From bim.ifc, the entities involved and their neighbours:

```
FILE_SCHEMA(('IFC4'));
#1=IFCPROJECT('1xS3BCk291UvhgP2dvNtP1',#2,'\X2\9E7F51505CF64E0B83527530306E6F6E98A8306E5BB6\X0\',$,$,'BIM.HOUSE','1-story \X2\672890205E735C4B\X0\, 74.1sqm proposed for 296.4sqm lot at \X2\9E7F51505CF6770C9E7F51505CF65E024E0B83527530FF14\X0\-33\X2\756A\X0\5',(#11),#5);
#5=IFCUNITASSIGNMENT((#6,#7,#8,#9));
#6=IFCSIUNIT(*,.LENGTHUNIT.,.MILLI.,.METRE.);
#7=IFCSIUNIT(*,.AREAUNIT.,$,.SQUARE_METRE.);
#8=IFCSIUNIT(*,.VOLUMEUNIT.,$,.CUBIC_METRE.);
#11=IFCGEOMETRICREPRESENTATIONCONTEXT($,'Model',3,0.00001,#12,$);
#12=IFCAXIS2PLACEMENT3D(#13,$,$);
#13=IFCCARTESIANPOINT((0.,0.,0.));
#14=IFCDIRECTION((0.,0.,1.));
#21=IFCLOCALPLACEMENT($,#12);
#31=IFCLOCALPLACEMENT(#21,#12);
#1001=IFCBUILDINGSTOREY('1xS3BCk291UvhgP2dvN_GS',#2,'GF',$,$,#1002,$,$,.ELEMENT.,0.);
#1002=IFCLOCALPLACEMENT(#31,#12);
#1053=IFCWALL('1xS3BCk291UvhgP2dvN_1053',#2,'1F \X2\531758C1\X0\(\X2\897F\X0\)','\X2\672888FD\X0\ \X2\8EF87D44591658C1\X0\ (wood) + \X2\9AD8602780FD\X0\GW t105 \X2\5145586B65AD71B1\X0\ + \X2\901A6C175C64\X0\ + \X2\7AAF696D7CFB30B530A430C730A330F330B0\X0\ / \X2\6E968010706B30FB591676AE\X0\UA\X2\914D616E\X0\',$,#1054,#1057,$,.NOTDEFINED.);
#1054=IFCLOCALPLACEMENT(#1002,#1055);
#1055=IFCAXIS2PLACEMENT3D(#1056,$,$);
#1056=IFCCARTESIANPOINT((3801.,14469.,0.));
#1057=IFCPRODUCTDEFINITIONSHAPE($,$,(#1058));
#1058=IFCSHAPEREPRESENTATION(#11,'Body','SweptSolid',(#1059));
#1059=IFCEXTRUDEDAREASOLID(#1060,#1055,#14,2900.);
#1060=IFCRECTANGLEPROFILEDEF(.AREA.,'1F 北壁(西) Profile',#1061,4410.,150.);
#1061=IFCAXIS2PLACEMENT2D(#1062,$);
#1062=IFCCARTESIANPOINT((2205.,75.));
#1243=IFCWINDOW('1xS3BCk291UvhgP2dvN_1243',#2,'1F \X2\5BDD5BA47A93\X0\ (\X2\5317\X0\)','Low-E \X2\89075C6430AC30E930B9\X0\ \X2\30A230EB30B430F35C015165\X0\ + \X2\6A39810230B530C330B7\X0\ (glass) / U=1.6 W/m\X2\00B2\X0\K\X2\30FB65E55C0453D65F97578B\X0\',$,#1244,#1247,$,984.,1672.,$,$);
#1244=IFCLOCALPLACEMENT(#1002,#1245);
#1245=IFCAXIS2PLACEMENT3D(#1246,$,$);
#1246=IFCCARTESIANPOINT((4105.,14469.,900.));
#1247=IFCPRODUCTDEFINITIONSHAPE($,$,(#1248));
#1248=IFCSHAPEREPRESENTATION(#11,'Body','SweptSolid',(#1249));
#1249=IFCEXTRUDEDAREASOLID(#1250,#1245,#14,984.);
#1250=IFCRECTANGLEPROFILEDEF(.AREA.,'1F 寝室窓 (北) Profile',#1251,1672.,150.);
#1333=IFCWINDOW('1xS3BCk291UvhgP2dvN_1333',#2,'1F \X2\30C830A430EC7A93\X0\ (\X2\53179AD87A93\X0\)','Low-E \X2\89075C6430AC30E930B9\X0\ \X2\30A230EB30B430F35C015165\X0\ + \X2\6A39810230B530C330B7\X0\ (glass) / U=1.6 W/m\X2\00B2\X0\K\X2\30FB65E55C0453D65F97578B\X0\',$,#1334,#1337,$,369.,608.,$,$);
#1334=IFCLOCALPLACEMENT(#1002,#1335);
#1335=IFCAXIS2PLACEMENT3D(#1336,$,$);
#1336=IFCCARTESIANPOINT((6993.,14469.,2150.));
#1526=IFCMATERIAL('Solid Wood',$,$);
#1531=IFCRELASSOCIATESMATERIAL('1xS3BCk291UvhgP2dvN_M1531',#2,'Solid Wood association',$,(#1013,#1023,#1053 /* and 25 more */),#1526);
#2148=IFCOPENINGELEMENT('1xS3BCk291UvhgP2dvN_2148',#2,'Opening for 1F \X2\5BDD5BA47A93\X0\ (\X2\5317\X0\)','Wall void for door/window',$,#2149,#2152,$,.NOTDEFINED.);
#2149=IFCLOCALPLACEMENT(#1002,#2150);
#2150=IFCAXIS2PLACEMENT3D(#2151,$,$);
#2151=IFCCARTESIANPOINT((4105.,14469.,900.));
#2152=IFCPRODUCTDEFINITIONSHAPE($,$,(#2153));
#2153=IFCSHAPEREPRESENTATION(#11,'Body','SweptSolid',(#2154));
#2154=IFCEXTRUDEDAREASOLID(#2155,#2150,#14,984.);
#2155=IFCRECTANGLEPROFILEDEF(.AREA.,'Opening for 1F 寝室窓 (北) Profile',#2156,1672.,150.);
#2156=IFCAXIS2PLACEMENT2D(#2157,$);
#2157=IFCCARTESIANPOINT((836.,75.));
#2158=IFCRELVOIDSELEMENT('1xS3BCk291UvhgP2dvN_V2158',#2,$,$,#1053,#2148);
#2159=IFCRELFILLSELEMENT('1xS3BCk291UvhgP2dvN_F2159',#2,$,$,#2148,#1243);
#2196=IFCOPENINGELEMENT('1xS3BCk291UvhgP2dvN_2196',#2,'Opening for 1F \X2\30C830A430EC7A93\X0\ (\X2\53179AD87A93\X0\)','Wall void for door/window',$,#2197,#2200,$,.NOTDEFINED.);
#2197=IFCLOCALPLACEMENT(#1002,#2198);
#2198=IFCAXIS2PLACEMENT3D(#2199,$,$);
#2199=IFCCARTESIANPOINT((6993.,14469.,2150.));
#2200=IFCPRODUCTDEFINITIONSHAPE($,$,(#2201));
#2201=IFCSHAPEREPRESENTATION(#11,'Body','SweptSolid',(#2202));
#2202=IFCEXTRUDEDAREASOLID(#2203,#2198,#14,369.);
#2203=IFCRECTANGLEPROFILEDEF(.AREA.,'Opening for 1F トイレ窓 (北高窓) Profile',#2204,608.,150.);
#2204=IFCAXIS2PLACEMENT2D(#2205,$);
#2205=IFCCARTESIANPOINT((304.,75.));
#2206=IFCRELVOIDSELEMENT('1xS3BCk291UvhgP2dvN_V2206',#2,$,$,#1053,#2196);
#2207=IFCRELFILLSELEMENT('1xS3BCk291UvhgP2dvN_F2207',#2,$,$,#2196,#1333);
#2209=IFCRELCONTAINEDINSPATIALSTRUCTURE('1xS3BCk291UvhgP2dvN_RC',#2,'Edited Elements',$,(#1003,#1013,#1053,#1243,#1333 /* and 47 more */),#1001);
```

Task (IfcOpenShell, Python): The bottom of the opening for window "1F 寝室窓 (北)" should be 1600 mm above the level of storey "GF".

```python
import numpy as np
import ifcopenshell
import ifcopenshell.api.geometry
import ifcopenshell.geom
import ifcopenshell.util.element
import ifcopenshell.util.placement
import ifcopenshell.util.shape
import ifcopenshell.util.unit

model = ifcopenshell.open("bim.ifc")
unit_scale = ifcopenshell.util.unit.calculate_unit_scale(model)

window = model.by_id(1243)
opening = window.FillsVoids[0].RelatingOpeningElement
storey = ifcopenshell.util.element.get_container(window, ifc_class="IfcBuildingStorey")
level = ifcopenshell.util.placement.get_local_placement(storey.ObjectPlacement)[2, 3]

# The opening's origin need not be at the sill, so measure its lowest point.
shape = ifcopenshell.geom.create_shape(ifcopenshell.geom.settings(), opening)
bottom = ifcopenshell.util.shape.get_shape_bottom_elevation(shape, shape.geometry) / unit_scale
dz = level + 1.6 / unit_scale - bottom

shift = np.array([0.0, 0.0, dz])
# The window is not placed relative to its opening, so move both.
for product in (opening, window):
    matrix = ifcopenshell.util.placement.get_local_placement(product.ObjectPlacement)
    matrix[:3, 3] += shift
    ifcopenshell.api.geometry.edit_object_placement(model, product=product, matrix=matrix, is_si=False)

print(f"moved by {dz * unit_scale:+.3f} m")

model.write("bim-out.ifc")
```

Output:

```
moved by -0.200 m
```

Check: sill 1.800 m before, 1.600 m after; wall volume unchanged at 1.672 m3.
